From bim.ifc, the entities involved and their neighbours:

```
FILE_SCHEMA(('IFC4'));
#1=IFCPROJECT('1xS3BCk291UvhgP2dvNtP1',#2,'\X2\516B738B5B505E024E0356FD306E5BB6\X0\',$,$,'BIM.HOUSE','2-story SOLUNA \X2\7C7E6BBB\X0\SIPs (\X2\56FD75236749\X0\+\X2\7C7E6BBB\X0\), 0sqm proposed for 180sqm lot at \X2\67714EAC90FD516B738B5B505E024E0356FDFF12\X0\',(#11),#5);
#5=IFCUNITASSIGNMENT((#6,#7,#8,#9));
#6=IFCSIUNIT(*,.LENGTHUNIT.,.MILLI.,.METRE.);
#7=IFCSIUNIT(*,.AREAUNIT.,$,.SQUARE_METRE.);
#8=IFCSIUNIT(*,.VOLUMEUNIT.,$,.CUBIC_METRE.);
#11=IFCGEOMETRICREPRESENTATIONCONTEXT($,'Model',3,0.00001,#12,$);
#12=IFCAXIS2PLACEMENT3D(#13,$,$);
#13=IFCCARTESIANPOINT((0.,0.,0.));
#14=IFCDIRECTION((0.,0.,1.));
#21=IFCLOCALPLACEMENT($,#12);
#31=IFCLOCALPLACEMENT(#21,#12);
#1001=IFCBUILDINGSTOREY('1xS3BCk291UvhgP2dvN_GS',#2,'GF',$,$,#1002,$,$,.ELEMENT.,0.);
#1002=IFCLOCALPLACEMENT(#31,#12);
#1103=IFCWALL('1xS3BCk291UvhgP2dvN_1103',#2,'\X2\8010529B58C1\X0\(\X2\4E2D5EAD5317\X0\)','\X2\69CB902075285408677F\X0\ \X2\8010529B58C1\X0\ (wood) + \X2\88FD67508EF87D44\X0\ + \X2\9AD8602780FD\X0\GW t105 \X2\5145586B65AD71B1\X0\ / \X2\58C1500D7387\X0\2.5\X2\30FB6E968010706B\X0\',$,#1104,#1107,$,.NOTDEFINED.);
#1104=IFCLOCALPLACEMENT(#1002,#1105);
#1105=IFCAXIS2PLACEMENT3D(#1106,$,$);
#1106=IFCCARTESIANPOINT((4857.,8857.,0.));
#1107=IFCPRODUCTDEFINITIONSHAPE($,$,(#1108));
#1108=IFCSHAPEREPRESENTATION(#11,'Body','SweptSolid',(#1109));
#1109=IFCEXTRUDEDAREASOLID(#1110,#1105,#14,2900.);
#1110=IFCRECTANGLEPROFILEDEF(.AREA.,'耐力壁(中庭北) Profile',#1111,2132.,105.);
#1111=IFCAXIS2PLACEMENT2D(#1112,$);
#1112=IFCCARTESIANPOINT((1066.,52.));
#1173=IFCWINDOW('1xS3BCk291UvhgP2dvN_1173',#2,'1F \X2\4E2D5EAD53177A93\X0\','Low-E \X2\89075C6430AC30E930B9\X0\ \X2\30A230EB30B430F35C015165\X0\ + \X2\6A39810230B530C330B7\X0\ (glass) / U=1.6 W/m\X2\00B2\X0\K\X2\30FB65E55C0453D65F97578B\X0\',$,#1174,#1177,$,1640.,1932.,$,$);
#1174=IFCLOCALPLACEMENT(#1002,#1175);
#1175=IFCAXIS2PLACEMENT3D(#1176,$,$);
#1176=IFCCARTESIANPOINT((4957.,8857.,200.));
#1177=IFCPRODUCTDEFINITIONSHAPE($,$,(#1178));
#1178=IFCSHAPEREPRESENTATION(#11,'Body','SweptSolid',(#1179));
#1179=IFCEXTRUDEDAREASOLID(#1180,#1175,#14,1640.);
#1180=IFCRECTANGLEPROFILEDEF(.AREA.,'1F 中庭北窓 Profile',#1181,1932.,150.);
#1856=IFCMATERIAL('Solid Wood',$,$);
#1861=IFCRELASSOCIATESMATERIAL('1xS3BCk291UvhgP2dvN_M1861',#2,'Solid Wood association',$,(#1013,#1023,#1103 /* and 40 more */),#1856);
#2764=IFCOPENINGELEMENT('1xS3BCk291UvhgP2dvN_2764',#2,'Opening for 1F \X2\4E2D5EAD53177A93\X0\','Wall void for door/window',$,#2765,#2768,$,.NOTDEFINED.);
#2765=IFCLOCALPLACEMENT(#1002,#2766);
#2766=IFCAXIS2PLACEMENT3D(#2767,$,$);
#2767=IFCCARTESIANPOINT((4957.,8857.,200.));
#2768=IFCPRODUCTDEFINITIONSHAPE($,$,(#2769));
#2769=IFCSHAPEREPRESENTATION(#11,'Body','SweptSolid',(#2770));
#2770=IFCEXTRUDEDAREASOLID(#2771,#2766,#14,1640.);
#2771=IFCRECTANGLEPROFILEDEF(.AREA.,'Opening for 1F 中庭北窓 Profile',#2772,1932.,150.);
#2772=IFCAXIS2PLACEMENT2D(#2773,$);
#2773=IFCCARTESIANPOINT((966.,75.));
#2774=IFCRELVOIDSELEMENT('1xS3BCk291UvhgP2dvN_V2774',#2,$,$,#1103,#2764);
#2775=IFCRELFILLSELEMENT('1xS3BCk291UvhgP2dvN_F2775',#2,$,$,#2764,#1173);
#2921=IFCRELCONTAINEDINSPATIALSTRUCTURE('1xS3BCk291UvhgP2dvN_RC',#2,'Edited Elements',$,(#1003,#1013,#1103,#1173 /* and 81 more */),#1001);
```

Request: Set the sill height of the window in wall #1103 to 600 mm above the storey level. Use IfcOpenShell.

```python
import numpy as np
import ifcopenshell
import ifcopenshell.api.geometry
import ifcopenshell.geom
import ifcopenshell.util.element
import ifcopenshell.util.placement
import ifcopenshell.util.shape
import ifcopenshell.util.unit

model = ifcopenshell.open("bim.ifc")
unit_scale = ifcopenshell.util.unit.calculate_unit_scale(model)

window = model.by_guid("1xS3BCk291UvhgP2dvN_1173")
opening = window.FillsVoids[0].RelatingOpeningElement
storey = ifcopenshell.util.element.get_container(window, ifc_class="IfcBuildingStorey")
level = ifcopenshell.util.placement.get_local_placement(storey.ObjectPlacement)[2, 3]

# The opening's origin need not be at the sill, so measure its lowest point.
shape = ifcopenshell.geom.create_shape(ifcopenshell.geom.settings(), opening)
bottom = ifcopenshell.util.shape.get_shape_bottom_elevation(shape, shape.geometry) / unit_scale
dz = level + 600.0 - bottom

shift = np.array([0.0, 0.0, dz])
# The window is not placed relative to its opening, so move both.
for product in (opening, window):
    matrix = ifcopenshell.util.placement.get_local_placement(product.ObjectPlacement)
    matrix[:3, 3] += shift
    ifcopenshell.api.geometry.edit_object_placement(model, product=product, matrix=matrix, is_si=False)

print(f"moved by {dz * unit_scale:+.3f} m")

model.write("bim_rev.ifc")
```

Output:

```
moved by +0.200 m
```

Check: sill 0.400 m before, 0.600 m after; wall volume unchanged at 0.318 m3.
